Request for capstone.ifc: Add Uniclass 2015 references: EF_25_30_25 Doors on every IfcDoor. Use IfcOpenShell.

First a look at what the model holds.

```python
import ifcopenshell

model = ifcopenshell.open("capstone.ifc")
print(model.schema)
print("classifications:", [c.Name for c in model.by_type("IfcClassification")])
for ifc_class in ("IfcDoor", "IfcRoof", "IfcStair", "IfcWall", "IfcWindow"):
    print(ifc_class, len(model.by_type(ifc_class)))
```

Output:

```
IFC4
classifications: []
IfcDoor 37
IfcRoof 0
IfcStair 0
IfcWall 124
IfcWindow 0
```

```python
import ifcopenshell
import ifcopenshell.api.classification

model = ifcopenshell.open("capstone.ifc")

system = ifcopenshell.api.classification.add_classification(model, classification="Uniclass 2015")

codes = {
    "IfcDoor": ("EF_25_30_25", "Doors"),
}
for ifc_class, (code, name) in codes.items():
    products = model.by_type(ifc_class)
    ifcopenshell.api.classification.add_reference(
        model, products=products, classification=system, identification=code, name=name
    )
    print(code, len(products))

model.write("capstone_edited.ifc")
```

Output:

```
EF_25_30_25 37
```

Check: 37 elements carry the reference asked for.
